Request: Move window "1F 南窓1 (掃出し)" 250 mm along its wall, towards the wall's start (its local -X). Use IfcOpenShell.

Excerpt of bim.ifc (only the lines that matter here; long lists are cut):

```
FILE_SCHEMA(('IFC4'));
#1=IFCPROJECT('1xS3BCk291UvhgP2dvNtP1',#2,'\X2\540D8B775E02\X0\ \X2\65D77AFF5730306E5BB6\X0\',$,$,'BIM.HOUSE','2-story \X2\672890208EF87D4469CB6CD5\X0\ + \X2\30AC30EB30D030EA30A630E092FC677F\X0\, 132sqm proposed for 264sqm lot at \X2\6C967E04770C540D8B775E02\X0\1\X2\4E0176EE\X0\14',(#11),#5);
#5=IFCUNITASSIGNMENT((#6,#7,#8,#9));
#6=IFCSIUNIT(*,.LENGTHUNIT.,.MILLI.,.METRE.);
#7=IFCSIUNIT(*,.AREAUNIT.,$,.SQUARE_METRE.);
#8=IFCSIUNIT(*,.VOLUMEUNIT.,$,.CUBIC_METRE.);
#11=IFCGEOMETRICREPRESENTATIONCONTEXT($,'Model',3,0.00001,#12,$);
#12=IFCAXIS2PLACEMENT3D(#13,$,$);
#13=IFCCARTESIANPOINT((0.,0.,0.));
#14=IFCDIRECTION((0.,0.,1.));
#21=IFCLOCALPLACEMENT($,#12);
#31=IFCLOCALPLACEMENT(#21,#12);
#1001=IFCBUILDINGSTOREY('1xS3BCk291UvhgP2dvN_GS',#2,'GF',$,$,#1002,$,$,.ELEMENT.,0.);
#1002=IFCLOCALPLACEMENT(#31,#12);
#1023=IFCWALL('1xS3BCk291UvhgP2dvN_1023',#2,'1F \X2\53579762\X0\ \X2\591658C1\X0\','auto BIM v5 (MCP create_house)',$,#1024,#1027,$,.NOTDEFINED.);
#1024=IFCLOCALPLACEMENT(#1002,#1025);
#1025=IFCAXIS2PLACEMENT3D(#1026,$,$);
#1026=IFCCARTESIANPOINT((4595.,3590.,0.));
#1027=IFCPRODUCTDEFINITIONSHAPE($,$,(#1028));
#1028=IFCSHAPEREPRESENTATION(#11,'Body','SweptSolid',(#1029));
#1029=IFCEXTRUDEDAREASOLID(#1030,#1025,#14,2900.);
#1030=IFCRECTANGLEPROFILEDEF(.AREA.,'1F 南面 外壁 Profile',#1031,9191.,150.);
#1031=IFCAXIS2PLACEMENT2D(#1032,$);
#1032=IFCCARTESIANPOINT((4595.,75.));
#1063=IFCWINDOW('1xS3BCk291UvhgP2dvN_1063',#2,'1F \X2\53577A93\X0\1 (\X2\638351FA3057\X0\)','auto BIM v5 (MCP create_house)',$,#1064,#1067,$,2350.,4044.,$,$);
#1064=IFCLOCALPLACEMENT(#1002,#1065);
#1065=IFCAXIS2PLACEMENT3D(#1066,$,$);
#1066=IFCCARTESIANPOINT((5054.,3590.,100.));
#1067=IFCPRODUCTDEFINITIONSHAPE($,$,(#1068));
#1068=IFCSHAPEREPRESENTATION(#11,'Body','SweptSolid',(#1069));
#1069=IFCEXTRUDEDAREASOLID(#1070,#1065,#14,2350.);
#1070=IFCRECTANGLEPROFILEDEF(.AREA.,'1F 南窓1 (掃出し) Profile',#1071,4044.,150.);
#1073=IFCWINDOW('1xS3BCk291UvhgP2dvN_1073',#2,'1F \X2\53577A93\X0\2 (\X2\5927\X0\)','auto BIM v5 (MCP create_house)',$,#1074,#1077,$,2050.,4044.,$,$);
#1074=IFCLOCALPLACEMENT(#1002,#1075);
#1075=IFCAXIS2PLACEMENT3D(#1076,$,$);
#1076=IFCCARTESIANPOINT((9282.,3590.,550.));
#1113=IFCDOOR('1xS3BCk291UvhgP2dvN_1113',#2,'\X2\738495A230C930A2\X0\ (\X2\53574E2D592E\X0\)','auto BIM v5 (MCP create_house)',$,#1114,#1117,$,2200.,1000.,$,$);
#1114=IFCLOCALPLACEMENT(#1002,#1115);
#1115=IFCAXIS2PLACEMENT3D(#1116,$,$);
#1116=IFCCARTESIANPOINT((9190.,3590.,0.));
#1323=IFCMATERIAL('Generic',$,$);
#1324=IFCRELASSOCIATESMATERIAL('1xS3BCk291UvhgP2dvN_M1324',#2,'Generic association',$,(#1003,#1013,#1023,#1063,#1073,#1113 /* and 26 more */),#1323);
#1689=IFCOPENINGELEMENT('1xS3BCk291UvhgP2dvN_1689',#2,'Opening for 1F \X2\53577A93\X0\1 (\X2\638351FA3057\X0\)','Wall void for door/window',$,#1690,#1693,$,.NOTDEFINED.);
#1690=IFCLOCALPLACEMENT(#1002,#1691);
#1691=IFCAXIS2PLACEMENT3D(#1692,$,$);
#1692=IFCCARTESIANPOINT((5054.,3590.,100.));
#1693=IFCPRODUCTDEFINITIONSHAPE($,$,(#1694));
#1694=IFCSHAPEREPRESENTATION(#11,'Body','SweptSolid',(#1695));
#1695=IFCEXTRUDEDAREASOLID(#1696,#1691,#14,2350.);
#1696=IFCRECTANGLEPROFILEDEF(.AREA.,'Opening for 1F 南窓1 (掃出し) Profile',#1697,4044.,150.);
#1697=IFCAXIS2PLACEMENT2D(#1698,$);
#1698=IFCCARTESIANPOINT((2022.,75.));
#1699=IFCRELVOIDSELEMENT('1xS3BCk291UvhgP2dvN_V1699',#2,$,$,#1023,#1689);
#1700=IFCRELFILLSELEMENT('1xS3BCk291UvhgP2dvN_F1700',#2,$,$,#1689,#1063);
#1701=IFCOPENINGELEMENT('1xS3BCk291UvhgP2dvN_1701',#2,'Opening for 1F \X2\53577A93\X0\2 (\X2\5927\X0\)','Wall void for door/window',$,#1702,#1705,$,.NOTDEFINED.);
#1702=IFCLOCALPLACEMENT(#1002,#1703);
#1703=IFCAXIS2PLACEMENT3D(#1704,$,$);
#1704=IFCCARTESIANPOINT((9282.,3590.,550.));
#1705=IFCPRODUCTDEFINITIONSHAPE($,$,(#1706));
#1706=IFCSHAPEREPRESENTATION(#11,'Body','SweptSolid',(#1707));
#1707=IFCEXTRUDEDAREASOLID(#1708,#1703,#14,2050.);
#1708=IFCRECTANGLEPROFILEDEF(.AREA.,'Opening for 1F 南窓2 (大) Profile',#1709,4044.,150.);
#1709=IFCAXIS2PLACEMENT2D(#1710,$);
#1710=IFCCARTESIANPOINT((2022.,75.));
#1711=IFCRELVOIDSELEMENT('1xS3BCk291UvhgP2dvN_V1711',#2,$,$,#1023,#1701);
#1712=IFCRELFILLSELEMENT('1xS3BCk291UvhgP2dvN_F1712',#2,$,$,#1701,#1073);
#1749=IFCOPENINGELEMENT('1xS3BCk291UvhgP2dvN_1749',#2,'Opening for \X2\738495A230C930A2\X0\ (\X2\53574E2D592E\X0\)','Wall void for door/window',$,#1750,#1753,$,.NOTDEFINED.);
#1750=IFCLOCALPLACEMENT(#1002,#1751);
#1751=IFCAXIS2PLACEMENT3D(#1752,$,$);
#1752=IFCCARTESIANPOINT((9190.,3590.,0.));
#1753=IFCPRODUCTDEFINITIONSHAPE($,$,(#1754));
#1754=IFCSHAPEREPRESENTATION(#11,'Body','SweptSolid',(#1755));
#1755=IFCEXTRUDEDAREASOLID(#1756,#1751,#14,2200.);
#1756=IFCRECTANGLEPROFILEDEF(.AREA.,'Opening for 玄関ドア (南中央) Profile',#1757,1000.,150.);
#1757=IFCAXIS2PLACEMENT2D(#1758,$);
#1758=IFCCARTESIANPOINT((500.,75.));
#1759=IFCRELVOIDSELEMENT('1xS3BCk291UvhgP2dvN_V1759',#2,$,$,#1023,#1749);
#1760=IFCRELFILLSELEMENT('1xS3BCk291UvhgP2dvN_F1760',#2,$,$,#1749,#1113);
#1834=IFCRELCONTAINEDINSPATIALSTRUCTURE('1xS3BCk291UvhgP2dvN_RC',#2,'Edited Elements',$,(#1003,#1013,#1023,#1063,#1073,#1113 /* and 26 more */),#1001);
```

```python
import ifcopenshell
import ifcopenshell.api.geometry
import ifcopenshell.util.placement
import ifcopenshell.util.unit

model = ifcopenshell.open("bim.ifc")
unit_scale = ifcopenshell.util.unit.calculate_unit_scale(model)

window = model.by_id(1063)
opening = window.FillsVoids[0].RelatingOpeningElement
wall = opening.VoidsElements[0].RelatingBuildingElement

wall_matrix = ifcopenshell.util.placement.get_local_placement(wall.ObjectPlacement)
shift = wall_matrix[:3, 0] * -0.25 / unit_scale
before = ifcopenshell.util.placement.get_local_placement(window.ObjectPlacement)[:3, 3].copy()

# The window is not placed relative to its opening, so move both.
for product in (opening, window):
    matrix = ifcopenshell.util.placement.get_local_placement(product.ObjectPlacement)
    matrix[:3, 3] += shift
    ifcopenshell.api.geometry.edit_object_placement(model, product=product, matrix=matrix, is_si=False)

after = ifcopenshell.util.placement.get_local_placement(window.ObjectPlacement)[:3, 3]
print("window moved by", (after - before).round(3) + 0.0)

model.write("bim_rev.ifc")
```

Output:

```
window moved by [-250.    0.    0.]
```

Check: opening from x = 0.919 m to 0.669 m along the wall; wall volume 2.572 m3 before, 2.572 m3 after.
